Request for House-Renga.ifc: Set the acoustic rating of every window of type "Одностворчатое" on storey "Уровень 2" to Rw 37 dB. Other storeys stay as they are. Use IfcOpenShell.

First a look at what the model holds.

```python
import ifcopenshell
import ifcopenshell.util.element

model = ifcopenshell.open("House-Renga.ifc")
print(model.schema)
storey = next(s for s in model.by_type("IfcBuildingStorey") if s.Name == "Уровень 2")
windows = [e for e in ifcopenshell.util.element.get_decomposition(storey) if e.is_a("IfcWindow")]
seen = {}
for e in windows:
    element_type = ifcopenshell.util.element.get_type(e)
    key = (element_type.Name if element_type != e and element_type else None, ifcopenshell.util.element.get_pset(e, "Pset_WindowCommon", "AcousticRating"))
    seen[key] = seen.get(key, 0) + 1
for (name, value), count in sorted(seen.items(), key=str):
    print(count, "x", name, "|", value)
```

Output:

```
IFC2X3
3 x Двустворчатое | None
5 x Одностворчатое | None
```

```python
import ifcopenshell
import ifcopenshell.api.pset
import ifcopenshell.util.element

model = ifcopenshell.open("House-Renga.ifc")

storey = next(s for s in model.by_type("IfcBuildingStorey") if s.Name == "Уровень 2")
windows = [e for e in ifcopenshell.util.element.get_decomposition(storey) if e.is_a("IfcWindow")]

count = 0
for e in windows:
    element_type = ifcopenshell.util.element.get_type(e)
    if element_type in (None, e) or element_type.Name != "Одностворчатое":
        continue
    # add_pset returns the element's existing set when there is one.
    pset = ifcopenshell.api.pset.add_pset(model, product=e, name="Pset_WindowCommon")
    ifcopenshell.api.pset.edit_pset(model, pset=pset, properties={"AcousticRating": "Rw 37 dB"})
    count += 1

print(count, "windows updated")

model.write("House-Renga_rev.ifc")
```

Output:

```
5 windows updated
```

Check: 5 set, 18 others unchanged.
